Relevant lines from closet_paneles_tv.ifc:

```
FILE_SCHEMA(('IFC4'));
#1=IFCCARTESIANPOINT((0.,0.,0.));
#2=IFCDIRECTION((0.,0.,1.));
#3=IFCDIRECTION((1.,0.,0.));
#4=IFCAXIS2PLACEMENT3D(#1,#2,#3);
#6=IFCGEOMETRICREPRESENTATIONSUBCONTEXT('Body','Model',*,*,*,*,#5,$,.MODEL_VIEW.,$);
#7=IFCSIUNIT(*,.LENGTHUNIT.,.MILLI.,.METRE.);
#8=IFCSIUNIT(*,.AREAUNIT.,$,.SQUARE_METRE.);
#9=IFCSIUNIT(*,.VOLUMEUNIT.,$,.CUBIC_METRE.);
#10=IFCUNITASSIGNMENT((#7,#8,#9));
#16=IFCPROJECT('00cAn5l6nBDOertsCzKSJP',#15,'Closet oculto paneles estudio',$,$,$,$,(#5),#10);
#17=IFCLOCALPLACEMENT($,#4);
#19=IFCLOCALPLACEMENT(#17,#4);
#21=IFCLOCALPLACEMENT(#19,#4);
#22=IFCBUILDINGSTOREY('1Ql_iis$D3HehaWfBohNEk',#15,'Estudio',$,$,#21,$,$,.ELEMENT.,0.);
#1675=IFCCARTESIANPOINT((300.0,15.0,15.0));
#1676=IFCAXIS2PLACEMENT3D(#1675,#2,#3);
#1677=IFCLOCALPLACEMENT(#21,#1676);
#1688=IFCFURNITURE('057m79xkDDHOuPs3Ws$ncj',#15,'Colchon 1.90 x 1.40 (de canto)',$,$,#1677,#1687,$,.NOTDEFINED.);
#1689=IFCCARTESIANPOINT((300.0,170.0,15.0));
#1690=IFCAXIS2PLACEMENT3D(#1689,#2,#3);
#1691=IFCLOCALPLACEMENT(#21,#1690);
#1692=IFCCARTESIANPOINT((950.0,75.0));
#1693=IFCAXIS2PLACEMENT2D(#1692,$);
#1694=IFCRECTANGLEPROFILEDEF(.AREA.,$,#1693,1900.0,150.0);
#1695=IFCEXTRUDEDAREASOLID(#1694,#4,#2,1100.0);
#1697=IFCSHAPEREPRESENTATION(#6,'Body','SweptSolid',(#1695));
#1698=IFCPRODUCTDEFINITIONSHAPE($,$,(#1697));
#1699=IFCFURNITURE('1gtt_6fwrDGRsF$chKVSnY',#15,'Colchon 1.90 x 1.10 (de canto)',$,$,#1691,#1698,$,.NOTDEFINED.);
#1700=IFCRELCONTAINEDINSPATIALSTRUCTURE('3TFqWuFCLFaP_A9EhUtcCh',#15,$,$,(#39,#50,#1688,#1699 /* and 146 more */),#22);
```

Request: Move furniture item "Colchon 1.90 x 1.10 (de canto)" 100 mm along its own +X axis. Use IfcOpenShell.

```python
import ifcopenshell
import ifcopenshell.api.geometry
import ifcopenshell.util.placement
import ifcopenshell.util.unit

model = ifcopenshell.open("closet_paneles_tv.ifc")
unit_scale = ifcopenshell.util.unit.calculate_unit_scale(model)

item = model.by_guid("1gtt_6fwrDGRsF$chKVSnY")
matrix = ifcopenshell.util.placement.get_local_placement(item.ObjectPlacement)
matrix[:3, 3] += matrix[:3, 0] * 0.1 / unit_scale
ifcopenshell.api.geometry.edit_object_placement(model, product=item, matrix=matrix, is_si=False)

print(ifcopenshell.util.placement.get_local_placement(item.ObjectPlacement).round(3) + 0.0)

model.write("closet_paneles_tv_rev.ifc")
```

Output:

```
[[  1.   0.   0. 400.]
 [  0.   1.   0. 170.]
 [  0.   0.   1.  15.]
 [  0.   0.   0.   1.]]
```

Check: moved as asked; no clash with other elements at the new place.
